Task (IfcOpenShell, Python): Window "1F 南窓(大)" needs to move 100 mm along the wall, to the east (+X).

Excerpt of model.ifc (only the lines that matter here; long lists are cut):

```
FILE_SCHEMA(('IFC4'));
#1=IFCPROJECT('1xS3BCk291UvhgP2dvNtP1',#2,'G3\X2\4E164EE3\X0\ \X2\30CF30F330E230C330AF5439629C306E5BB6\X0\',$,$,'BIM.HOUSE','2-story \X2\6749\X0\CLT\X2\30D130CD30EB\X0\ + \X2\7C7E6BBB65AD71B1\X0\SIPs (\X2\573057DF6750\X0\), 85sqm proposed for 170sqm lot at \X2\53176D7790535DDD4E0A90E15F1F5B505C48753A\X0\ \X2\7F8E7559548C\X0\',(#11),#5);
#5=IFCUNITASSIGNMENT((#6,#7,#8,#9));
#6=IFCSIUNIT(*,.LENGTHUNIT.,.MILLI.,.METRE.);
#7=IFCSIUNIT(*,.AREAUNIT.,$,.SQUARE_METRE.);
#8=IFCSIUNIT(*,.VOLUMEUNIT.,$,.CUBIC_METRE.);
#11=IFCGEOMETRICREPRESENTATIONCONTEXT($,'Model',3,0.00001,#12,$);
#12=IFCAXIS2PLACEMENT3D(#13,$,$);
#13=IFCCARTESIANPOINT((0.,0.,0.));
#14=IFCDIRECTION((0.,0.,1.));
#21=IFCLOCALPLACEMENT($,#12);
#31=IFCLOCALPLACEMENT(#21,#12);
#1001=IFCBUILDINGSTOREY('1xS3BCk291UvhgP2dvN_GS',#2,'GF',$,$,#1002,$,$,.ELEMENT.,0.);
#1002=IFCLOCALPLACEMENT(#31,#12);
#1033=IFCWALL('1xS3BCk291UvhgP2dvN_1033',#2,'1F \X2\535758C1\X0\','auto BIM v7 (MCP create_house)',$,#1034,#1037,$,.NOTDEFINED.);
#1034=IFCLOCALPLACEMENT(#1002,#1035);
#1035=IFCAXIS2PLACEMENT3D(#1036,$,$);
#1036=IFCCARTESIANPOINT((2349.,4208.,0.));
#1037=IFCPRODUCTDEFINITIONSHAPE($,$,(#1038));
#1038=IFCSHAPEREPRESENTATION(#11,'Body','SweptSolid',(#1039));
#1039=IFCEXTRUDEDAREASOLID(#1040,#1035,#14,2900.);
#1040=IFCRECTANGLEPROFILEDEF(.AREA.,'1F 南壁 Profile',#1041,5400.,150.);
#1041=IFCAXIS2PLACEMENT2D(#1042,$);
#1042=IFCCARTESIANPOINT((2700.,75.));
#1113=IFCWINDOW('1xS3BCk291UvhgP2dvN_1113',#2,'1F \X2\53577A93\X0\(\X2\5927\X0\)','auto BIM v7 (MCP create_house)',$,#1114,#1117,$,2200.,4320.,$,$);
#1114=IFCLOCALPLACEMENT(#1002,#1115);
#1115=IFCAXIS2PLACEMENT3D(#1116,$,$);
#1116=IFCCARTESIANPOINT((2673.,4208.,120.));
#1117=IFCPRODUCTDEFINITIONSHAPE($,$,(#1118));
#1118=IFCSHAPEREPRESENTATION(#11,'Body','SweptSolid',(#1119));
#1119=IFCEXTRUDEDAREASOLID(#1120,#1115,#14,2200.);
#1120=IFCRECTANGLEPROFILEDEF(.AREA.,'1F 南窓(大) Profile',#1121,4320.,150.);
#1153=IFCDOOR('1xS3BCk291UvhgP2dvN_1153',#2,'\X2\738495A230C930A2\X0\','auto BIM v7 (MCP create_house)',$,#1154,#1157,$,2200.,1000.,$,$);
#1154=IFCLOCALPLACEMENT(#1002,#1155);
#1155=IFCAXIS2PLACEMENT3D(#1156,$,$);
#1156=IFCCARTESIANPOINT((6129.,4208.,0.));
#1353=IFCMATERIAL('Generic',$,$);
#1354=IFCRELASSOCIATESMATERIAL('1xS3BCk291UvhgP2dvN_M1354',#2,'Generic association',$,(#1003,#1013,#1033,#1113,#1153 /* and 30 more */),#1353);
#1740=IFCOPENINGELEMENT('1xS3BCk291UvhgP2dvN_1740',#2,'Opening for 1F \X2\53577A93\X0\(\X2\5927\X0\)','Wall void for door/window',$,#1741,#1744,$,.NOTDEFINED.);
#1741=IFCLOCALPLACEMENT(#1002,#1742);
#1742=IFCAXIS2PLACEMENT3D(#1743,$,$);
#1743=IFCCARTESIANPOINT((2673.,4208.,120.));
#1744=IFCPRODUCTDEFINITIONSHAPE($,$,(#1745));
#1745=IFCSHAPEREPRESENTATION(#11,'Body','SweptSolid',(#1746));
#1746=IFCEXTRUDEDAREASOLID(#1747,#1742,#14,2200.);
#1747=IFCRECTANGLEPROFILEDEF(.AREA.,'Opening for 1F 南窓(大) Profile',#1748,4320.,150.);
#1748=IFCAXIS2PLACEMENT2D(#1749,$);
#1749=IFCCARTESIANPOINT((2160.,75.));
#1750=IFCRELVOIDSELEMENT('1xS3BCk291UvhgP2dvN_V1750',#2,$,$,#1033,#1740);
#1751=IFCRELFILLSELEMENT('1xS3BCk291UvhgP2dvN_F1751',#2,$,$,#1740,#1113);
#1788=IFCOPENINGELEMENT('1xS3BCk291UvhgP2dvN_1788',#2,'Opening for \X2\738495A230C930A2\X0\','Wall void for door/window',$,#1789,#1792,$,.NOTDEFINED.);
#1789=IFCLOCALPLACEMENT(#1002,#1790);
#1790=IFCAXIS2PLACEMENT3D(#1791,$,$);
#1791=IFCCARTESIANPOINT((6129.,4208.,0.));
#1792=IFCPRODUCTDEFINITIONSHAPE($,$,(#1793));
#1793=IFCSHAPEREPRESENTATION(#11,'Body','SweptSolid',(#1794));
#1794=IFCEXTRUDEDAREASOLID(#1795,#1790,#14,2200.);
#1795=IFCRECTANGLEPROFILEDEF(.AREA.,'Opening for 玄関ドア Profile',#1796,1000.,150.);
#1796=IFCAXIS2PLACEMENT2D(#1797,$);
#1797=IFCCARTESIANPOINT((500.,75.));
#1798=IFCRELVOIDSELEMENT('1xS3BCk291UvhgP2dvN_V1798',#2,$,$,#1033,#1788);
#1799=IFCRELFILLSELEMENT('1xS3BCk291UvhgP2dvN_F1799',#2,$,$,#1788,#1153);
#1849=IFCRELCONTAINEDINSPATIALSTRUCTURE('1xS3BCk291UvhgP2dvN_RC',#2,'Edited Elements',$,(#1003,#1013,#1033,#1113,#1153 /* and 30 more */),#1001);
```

```python
import ifcopenshell
import ifcopenshell.api.geometry
import ifcopenshell.util.placement
import ifcopenshell.util.unit

model = ifcopenshell.open("model.ifc")
unit_scale = ifcopenshell.util.unit.calculate_unit_scale(model)

window = model.by_id(1113)
opening = window.FillsVoids[0].RelatingOpeningElement
wall = opening.VoidsElements[0].RelatingBuildingElement

wall_matrix = ifcopenshell.util.placement.get_local_placement(wall.ObjectPlacement)
shift = wall_matrix[:3, 0] * 0.1 / unit_scale
before = ifcopenshell.util.placement.get_local_placement(window.ObjectPlacement)[:3, 3].copy()

# The window is not placed relative to its opening, so move both.
for product in (opening, window):
    matrix = ifcopenshell.util.placement.get_local_placement(product.ObjectPlacement)
    matrix[:3, 3] += shift
    ifcopenshell.api.geometry.edit_object_placement(model, product=product, matrix=matrix, is_si=False)

after = ifcopenshell.util.placement.get_local_placement(window.ObjectPlacement)[:3, 3]
print("window moved by", (after - before).round(3) + 0.0)

model.write("model-out.ifc")
```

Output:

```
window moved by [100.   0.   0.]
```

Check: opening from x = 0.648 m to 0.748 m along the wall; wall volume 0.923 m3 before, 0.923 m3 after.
